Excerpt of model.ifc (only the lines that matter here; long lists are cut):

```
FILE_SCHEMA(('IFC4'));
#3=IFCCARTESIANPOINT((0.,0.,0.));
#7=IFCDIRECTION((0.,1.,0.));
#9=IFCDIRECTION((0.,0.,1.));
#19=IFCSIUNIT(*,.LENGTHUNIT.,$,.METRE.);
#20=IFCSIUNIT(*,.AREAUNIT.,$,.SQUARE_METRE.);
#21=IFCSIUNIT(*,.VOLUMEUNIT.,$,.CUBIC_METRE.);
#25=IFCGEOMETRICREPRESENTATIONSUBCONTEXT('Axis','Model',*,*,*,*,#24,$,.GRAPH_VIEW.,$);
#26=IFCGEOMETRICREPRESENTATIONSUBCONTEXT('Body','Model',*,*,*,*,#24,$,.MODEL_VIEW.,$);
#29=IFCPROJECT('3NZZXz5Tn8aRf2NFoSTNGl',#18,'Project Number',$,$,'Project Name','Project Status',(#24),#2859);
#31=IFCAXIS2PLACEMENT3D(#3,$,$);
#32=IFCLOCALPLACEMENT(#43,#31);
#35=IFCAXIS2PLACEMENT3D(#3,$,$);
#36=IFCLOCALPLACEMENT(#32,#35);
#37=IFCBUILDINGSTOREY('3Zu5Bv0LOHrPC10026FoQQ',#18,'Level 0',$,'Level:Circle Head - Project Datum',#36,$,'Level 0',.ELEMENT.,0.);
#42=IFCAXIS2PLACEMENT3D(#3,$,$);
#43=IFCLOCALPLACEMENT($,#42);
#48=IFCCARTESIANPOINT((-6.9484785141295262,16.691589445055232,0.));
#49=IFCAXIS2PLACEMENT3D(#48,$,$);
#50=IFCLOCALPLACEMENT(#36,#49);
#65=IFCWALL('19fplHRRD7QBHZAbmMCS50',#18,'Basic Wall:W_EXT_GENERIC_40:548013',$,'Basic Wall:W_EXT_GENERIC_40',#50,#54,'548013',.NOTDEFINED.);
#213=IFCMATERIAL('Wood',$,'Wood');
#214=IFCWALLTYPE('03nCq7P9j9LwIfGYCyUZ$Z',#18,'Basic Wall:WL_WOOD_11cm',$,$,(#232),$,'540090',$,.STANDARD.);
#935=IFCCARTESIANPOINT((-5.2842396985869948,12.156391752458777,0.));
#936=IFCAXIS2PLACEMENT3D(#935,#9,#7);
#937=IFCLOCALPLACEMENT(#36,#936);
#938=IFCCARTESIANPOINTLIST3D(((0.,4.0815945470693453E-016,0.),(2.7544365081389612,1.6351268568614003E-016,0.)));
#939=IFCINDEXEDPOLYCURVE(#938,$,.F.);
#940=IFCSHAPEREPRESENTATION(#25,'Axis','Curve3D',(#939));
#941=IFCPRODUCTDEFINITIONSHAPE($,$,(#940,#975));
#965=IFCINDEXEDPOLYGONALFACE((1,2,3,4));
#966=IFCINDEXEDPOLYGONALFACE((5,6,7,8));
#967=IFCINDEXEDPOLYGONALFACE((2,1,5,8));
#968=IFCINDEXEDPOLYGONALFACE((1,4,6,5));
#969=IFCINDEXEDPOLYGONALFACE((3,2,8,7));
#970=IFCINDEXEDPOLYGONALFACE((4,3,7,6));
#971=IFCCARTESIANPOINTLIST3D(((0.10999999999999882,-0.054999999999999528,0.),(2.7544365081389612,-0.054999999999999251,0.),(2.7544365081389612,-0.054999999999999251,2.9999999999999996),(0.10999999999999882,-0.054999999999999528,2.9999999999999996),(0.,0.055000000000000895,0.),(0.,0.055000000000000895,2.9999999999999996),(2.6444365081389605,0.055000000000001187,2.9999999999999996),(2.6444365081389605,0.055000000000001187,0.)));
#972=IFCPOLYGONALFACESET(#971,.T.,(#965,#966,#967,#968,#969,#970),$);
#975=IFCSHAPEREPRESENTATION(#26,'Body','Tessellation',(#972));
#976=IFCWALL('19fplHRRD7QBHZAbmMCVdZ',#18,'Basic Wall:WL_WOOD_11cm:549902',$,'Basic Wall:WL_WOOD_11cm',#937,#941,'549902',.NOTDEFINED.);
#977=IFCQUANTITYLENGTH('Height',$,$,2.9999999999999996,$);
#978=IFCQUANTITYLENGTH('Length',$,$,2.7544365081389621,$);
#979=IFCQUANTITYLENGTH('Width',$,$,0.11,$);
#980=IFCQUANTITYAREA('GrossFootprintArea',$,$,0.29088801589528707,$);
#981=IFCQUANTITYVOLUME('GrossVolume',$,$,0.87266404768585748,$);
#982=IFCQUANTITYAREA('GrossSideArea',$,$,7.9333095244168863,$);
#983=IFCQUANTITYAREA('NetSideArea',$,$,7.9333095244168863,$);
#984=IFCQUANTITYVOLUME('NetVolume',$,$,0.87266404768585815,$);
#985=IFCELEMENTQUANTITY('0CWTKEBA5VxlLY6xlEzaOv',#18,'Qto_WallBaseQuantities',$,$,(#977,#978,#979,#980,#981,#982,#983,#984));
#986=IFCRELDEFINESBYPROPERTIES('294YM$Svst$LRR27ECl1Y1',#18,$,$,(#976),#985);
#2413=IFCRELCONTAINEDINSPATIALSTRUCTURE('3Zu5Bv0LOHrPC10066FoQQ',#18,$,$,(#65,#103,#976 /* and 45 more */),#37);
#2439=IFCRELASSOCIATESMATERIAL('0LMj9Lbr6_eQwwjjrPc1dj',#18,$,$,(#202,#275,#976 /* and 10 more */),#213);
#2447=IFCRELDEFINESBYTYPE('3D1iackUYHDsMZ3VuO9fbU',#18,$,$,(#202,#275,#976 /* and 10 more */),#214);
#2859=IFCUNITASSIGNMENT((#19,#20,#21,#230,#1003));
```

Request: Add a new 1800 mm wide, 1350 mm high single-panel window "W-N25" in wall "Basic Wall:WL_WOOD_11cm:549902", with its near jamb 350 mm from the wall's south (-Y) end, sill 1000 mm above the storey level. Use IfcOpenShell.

```python
import numpy as np
import ifcopenshell
import ifcopenshell.api.feature
import ifcopenshell.api.geometry
import ifcopenshell.api.pset
import ifcopenshell.api.root
import ifcopenshell.api.spatial
import ifcopenshell.geom
import ifcopenshell.util.element
import ifcopenshell.util.placement
import ifcopenshell.util.representation
import ifcopenshell.util.shape
import ifcopenshell.util.unit

model = ifcopenshell.open("model.ifc")
unit_scale = ifcopenshell.util.unit.calculate_unit_scale(model)
area_scale = ifcopenshell.util.unit.calculate_unit_scale(model, "AREAUNIT")
volume_scale = ifcopenshell.util.unit.calculate_unit_scale(model, "VOLUMEUNIT")
settings = ifcopenshell.geom.settings()


def volume(element):
    """Net volume in cubic metres, openings subtracted."""
    shape = ifcopenshell.geom.create_shape(settings, element)
    return ifcopenshell.util.shape.get_volume(shape.geometry)


wall = model.by_id(976)
storey = ifcopenshell.util.element.get_container(wall, ifc_class="IfcBuildingStorey")
context = ifcopenshell.util.representation.get_context(model, "Model", "Body", "MODEL_VIEW")
before = volume(wall)

width, height, from_end, sill = 1.8, 1.35, 0.35, 1  # metres

# The wall runs along its own X axis, and the end named is its -X end.
wall_shape = ifcopenshell.geom.create_shape(settings, wall)
x, y, z = ifcopenshell.util.shape.get_vertices(wall_shape.geometry).T
start = x.min() + from_end
face, thickness = float(y.min()), float(y.max() - y.min())
wall_matrix = ifcopenshell.util.placement.get_local_placement(wall.ObjectPlacement)
level = ifcopenshell.util.placement.get_local_placement(storey.ObjectPlacement)[2, 3]


def in_wall(x, y):
    """Placement at x, y metres in the wall's axes, at sill height."""
    matrix = wall_matrix.copy()
    matrix[:, 3] = wall_matrix @ np.array([x / unit_scale, y / unit_scale, 0.0, 1.0])
    matrix[2, 3] = level + sill / unit_scale
    return matrix


# Opening: a box that overshoots both wall faces by 50 mm.
opening = ifcopenshell.api.root.create_entity(model, ifc_class="IfcOpeningElement", predefined_type="OPENING")
box = ifcopenshell.api.geometry.add_wall_representation(
    model, context=context, length=width, height=height, thickness=thickness + 0.1
)
ifcopenshell.api.geometry.assign_representation(model, product=opening, representation=box)
ifcopenshell.api.geometry.edit_object_placement(model, product=opening, matrix=in_wall(start, face - 0.05), is_si=False)
ifcopenshell.api.feature.add_feature(model, feature=opening, element=wall)

window = ifcopenshell.api.root.create_entity(model, ifc_class="IfcWindow", name="W-N25", predefined_type="WINDOW")
window.OverallWidth, window.OverallHeight = width / unit_scale, height / unit_scale
window.PartitioningType = "SINGLE_PANEL"
body = ifcopenshell.api.geometry.add_window_representation(
    model,
    context=context,
    overall_width=window.OverallWidth,
    overall_height=window.OverallHeight,
    partition_type="SINGLE_PANEL",
)
ifcopenshell.api.geometry.assign_representation(model, product=window, representation=body)
ifcopenshell.api.spatial.assign_container(model, products=[window], relating_structure=storey)
ifcopenshell.api.feature.add_filling(model, opening=opening, element=window)

# Centre the window in the wall's thickness.
ifcopenshell.api.geometry.edit_object_placement(model, product=window, matrix=in_wall(start, face), is_si=False)
window_shape = ifcopenshell.geom.create_shape(settings, window)
depth = ifcopenshell.util.shape.get_vertices(window_shape.geometry)[:, 1]
offset = face + thickness / 2 - (depth.min() + depth.max()) / 2
ifcopenshell.api.geometry.edit_object_placement(model, product=window, matrix=in_wall(start, offset), is_si=False)

after = volume(wall)

# Update the wall's stored quantities.
qto = model.by_id(ifcopenshell.util.element.get_pset(wall, "Qto_WallBaseQuantities", should_inherit=False)["id"])
ifcopenshell.api.pset.edit_qto(model, qto=qto, properties={
    "NetSideArea": after / thickness / area_scale,
    "NetVolume": after / volume_scale,
})

print(f"wall volume {before:.3f} -> {after:.3f} m3")

model.write("model_edited.ifc")
```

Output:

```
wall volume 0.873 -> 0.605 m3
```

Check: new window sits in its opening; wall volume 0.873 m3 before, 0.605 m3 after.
